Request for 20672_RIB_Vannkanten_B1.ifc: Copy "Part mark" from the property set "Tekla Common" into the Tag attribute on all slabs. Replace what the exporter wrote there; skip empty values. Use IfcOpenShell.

First a look at what the model holds.

```python
import ifcopenshell
import ifcopenshell.util.element

model = ifcopenshell.open("20672_RIB_Vannkanten_B1.ifc")
print(model.schema)
slabs = model.by_type("IfcSlab")
print(len(slabs), "slabs")
for e in slabs[:8]:
    source = ifcopenshell.util.element.get_pset(e, "Tekla Common", "Part mark")
    target = e.Tag
    print(e.id(), repr(source), repr(target), sep=" | ")
```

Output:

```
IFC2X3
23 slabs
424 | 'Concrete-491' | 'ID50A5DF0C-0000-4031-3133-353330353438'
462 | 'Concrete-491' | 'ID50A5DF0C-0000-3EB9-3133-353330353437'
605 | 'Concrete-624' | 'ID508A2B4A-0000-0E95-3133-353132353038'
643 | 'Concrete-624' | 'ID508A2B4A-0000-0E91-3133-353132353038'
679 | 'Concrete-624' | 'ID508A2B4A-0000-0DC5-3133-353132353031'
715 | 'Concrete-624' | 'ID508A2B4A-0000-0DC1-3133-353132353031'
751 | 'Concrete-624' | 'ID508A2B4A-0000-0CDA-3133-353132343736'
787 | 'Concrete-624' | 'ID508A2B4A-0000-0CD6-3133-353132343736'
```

```python
import ifcopenshell
import ifcopenshell.util.element

model = ifcopenshell.open("20672_RIB_Vannkanten_B1.ifc")

count = 0
for e in model.by_type("IfcSlab"):
    value = ifcopenshell.util.element.get_pset(e, "Tekla Common", "Part mark")
    current = e.Tag
    if not value or not value.strip() or current == value:
        continue
    e.Tag = value
    count += 1

print(count, "slabs updated")

model.write("20672_RIB_Vannkanten_B1_rev.ifc")
```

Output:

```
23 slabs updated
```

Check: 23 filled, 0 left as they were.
